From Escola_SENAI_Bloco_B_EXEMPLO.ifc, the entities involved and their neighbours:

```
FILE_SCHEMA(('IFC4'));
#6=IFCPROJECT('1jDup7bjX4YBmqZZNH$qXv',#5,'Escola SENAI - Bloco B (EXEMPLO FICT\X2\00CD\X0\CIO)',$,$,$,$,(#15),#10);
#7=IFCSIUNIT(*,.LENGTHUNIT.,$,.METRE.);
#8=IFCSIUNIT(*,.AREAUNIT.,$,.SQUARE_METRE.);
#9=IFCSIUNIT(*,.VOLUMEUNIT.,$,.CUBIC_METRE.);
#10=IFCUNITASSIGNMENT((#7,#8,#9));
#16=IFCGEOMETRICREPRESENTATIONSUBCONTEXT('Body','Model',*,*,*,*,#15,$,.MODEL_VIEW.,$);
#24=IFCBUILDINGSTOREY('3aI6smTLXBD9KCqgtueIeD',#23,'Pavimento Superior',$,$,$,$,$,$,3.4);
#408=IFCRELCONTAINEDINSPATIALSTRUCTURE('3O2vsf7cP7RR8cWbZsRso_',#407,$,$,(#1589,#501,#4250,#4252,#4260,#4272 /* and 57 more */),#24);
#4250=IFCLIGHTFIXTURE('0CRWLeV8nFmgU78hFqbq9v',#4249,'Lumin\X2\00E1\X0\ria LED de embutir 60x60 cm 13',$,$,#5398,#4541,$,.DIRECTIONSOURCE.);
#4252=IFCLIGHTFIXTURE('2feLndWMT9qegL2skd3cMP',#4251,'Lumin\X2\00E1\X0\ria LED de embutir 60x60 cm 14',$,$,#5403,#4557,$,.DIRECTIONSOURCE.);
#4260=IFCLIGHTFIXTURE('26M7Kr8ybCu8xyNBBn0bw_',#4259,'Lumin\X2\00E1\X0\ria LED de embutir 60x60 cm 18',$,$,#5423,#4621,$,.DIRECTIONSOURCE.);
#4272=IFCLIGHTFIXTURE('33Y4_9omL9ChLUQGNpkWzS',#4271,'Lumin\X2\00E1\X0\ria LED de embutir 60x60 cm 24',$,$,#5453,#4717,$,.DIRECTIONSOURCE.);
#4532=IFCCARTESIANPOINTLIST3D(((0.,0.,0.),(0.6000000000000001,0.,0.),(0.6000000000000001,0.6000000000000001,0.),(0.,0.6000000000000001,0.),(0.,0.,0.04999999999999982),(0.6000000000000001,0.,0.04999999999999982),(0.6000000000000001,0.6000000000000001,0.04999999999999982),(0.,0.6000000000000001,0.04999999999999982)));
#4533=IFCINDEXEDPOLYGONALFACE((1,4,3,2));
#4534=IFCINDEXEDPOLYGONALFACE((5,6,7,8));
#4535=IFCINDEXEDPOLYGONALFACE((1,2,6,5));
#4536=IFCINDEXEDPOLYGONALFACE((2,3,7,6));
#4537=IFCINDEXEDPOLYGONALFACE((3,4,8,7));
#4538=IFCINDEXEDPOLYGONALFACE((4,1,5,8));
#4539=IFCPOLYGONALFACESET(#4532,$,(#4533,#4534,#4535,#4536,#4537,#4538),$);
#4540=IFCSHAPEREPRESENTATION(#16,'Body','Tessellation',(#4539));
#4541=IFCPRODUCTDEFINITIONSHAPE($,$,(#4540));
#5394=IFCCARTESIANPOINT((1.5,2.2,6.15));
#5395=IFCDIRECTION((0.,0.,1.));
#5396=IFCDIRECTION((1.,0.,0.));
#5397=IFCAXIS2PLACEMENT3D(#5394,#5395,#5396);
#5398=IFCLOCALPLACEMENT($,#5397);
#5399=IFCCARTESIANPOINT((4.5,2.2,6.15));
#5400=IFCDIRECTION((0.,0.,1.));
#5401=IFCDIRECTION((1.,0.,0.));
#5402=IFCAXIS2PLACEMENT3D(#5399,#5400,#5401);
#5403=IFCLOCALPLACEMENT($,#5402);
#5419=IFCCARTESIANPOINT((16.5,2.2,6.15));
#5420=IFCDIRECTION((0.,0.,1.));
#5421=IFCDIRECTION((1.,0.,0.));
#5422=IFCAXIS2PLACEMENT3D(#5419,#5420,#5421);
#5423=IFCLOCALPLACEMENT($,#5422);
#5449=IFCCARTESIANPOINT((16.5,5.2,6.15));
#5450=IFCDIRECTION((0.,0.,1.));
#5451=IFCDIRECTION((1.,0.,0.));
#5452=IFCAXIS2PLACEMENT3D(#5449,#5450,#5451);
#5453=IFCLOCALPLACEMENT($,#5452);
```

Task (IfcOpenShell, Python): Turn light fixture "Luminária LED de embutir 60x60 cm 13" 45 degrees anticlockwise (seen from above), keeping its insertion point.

```python
import ifcopenshell
import ifcopenshell.api.geometry
import ifcopenshell.util.placement

model = ifcopenshell.open("Escola_SENAI_Bloco_B_EXEMPLO.ifc")

item = model.by_guid("0CRWLeV8nFmgU78hFqbq9v")
matrix = ifcopenshell.util.placement.get_local_placement(item.ObjectPlacement)
matrix = matrix @ ifcopenshell.util.placement.rotation(45, "Z")
ifcopenshell.api.geometry.edit_object_placement(model, product=item, matrix=matrix, is_si=False)

print(ifcopenshell.util.placement.get_local_placement(item.ObjectPlacement).round(3) + 0.0)

model.write("Escola_SENAI_Bloco_B_EXEMPLO_edited.ifc")
```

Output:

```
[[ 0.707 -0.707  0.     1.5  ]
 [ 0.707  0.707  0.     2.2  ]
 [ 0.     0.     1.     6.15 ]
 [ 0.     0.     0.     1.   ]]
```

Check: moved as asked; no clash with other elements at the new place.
